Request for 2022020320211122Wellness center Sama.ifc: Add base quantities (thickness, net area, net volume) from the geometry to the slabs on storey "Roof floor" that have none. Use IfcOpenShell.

First a look at what the model holds.

```python
import ifcopenshell
import ifcopenshell.util.element
import ifcopenshell.util.unit

model = ifcopenshell.open("2022020320211122Wellness center Sama.ifc")
print(model.schema)
for unit_type in ("LENGTHUNIT", "AREAUNIT", "VOLUMEUNIT"):
    print(unit_type, ifcopenshell.util.unit.calculate_unit_scale(model, unit_type))
storey = next(s for s in model.by_type("IfcBuildingStorey") if s.Name == "Roof floor")
slabs = [e for e in ifcopenshell.util.element.get_decomposition(storey) if e.is_a("IfcSlab")]
for e in sorted(slabs, key=lambda e: e.id()):
    print(e.id(), e.is_a(), e.Name, list(ifcopenshell.util.element.get_psets(e, qtos_only=True)), sep=" | ")
```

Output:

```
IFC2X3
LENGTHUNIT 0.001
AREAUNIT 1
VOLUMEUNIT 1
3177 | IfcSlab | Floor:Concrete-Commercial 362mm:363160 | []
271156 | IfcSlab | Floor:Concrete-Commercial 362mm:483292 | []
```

```python
import ifcopenshell
import ifcopenshell.api.pset
import ifcopenshell.geom
import ifcopenshell.util.element
import ifcopenshell.util.shape
import ifcopenshell.util.unit

model = ifcopenshell.open("2022020320211122Wellness center Sama.ifc")
unit_scale = ifcopenshell.util.unit.calculate_unit_scale(model)
area_scale = ifcopenshell.util.unit.calculate_unit_scale(model, "AREAUNIT")
volume_scale = ifcopenshell.util.unit.calculate_unit_scale(model, "VOLUMEUNIT")
settings = ifcopenshell.geom.settings()

storey = next(s for s in model.by_type("IfcBuildingStorey") if s.Name == "Roof floor")
slabs = [e for e in ifcopenshell.util.element.get_decomposition(storey) if e.is_a("IfcSlab")]

for e in sorted(slabs, key=lambda e: e.id()):
    if ifcopenshell.util.element.get_psets(e, qtos_only=True, should_inherit=False):
        continue
    # Geometry comes back in metres, in the element's own axes.
    shape = ifcopenshell.geom.create_shape(settings, e)
    values = {
        "Width": ifcopenshell.util.shape.get_z(shape.geometry) / unit_scale,
        "NetArea": ifcopenshell.util.shape.get_footprint_area(shape.geometry) / area_scale,
        "NetVolume": ifcopenshell.util.shape.get_volume(shape.geometry) / volume_scale,
    }
    qto = ifcopenshell.api.pset.add_qto(model, product=e, name="BaseQuantities")
    ifcopenshell.api.pset.edit_qto(model, qto=qto, properties=values)
    print(e.id(), {k: round(v, 3) for k, v in values.items()})

model.write("2022020320211122Wellness center Sama_rev.ifc")
```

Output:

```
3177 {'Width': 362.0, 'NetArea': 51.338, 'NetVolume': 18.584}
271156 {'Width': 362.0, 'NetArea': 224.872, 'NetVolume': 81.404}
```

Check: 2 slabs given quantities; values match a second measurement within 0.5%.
